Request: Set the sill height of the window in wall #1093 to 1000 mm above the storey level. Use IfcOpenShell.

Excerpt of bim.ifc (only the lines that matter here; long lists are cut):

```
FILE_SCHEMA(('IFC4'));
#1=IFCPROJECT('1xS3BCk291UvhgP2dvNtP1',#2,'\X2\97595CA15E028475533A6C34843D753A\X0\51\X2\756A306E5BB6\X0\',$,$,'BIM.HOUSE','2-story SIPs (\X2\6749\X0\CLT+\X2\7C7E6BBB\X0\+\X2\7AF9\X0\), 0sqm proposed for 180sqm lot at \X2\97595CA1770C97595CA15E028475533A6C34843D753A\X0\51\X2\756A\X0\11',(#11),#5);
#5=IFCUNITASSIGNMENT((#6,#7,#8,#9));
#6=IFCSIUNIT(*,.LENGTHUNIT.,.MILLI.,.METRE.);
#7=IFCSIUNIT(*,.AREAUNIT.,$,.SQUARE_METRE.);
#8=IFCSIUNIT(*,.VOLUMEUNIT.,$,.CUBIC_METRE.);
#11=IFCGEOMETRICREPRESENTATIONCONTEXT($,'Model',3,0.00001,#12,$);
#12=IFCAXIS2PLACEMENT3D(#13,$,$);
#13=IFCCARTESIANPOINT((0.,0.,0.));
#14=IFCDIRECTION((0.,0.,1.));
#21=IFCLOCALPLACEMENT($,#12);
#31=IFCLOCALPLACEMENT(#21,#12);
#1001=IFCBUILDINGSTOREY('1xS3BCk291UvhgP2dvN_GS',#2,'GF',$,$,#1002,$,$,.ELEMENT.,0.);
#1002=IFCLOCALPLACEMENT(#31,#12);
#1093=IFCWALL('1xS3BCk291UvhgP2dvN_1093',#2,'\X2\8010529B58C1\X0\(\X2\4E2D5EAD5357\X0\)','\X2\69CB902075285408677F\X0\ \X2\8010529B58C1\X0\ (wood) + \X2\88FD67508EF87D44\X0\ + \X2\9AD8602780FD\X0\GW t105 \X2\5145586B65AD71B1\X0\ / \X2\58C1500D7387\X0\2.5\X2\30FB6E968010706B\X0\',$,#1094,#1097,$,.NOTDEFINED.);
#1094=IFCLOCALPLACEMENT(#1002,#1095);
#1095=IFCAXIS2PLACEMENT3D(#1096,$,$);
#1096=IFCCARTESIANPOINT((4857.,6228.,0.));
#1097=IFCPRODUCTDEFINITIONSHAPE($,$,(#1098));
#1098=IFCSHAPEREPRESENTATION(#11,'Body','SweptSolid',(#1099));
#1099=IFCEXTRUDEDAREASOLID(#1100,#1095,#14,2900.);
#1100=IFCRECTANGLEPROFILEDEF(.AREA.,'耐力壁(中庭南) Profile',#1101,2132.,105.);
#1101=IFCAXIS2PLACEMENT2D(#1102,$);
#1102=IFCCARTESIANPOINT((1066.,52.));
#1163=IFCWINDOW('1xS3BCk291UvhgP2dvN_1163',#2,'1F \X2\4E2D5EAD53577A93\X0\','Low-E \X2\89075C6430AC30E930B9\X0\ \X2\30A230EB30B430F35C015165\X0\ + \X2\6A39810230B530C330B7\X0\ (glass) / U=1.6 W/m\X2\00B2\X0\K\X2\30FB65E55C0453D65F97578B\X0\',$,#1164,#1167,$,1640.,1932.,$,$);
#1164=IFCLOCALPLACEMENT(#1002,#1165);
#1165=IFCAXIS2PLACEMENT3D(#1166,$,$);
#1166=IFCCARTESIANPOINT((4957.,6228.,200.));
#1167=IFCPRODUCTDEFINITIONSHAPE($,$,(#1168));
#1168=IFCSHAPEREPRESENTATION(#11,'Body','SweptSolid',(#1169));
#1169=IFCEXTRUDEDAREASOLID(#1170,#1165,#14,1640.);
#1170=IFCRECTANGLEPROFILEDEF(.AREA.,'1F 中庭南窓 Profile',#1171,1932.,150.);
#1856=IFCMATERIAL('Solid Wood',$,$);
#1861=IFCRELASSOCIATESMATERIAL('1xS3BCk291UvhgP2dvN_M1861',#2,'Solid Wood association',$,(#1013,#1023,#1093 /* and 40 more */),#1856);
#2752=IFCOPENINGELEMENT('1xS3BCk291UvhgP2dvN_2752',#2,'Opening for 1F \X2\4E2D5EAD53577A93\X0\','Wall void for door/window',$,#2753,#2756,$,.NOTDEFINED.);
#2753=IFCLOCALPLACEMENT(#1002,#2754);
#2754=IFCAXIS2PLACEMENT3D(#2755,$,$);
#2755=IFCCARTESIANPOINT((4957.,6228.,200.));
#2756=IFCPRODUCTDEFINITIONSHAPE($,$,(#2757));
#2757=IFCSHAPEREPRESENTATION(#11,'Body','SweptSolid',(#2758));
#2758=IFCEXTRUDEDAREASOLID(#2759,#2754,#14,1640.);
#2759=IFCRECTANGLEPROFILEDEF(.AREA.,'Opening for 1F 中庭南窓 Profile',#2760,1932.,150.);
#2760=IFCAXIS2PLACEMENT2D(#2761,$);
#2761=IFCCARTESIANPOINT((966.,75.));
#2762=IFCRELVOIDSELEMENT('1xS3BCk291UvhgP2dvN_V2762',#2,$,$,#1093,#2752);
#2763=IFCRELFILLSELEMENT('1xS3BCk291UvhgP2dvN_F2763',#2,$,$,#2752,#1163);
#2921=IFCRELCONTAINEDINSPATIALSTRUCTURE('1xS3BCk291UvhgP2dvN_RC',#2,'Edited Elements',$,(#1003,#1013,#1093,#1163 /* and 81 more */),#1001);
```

```python
import numpy as np
import ifcopenshell
import ifcopenshell.api.geometry
import ifcopenshell.geom
import ifcopenshell.util.element
import ifcopenshell.util.placement
import ifcopenshell.util.shape
import ifcopenshell.util.unit

model = ifcopenshell.open("bim.ifc")
unit_scale = ifcopenshell.util.unit.calculate_unit_scale(model)

window = model.by_id(1163)
opening = window.FillsVoids[0].RelatingOpeningElement
storey = ifcopenshell.util.element.get_container(window, ifc_class="IfcBuildingStorey")
level = ifcopenshell.util.placement.get_local_placement(storey.ObjectPlacement)[2, 3]

# The opening's origin need not be at the sill, so measure its lowest point.
shape = ifcopenshell.geom.create_shape(ifcopenshell.geom.settings(), opening)
bottom = ifcopenshell.util.shape.get_shape_bottom_elevation(shape, shape.geometry) / unit_scale
dz = level + 1 / unit_scale - bottom

shift = np.array([0.0, 0.0, dz])
# The window is not placed relative to its opening, so move both.
for product in (opening, window):
    matrix = ifcopenshell.util.placement.get_local_placement(product.ObjectPlacement)
    matrix[:3, 3] += shift
    ifcopenshell.api.geometry.edit_object_placement(model, product=product, matrix=matrix, is_si=False)

print(f"moved by {dz * unit_scale:+.3f} m")

model.write("bim-out.ifc")
```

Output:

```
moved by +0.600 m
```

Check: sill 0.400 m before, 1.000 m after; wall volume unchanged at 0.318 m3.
